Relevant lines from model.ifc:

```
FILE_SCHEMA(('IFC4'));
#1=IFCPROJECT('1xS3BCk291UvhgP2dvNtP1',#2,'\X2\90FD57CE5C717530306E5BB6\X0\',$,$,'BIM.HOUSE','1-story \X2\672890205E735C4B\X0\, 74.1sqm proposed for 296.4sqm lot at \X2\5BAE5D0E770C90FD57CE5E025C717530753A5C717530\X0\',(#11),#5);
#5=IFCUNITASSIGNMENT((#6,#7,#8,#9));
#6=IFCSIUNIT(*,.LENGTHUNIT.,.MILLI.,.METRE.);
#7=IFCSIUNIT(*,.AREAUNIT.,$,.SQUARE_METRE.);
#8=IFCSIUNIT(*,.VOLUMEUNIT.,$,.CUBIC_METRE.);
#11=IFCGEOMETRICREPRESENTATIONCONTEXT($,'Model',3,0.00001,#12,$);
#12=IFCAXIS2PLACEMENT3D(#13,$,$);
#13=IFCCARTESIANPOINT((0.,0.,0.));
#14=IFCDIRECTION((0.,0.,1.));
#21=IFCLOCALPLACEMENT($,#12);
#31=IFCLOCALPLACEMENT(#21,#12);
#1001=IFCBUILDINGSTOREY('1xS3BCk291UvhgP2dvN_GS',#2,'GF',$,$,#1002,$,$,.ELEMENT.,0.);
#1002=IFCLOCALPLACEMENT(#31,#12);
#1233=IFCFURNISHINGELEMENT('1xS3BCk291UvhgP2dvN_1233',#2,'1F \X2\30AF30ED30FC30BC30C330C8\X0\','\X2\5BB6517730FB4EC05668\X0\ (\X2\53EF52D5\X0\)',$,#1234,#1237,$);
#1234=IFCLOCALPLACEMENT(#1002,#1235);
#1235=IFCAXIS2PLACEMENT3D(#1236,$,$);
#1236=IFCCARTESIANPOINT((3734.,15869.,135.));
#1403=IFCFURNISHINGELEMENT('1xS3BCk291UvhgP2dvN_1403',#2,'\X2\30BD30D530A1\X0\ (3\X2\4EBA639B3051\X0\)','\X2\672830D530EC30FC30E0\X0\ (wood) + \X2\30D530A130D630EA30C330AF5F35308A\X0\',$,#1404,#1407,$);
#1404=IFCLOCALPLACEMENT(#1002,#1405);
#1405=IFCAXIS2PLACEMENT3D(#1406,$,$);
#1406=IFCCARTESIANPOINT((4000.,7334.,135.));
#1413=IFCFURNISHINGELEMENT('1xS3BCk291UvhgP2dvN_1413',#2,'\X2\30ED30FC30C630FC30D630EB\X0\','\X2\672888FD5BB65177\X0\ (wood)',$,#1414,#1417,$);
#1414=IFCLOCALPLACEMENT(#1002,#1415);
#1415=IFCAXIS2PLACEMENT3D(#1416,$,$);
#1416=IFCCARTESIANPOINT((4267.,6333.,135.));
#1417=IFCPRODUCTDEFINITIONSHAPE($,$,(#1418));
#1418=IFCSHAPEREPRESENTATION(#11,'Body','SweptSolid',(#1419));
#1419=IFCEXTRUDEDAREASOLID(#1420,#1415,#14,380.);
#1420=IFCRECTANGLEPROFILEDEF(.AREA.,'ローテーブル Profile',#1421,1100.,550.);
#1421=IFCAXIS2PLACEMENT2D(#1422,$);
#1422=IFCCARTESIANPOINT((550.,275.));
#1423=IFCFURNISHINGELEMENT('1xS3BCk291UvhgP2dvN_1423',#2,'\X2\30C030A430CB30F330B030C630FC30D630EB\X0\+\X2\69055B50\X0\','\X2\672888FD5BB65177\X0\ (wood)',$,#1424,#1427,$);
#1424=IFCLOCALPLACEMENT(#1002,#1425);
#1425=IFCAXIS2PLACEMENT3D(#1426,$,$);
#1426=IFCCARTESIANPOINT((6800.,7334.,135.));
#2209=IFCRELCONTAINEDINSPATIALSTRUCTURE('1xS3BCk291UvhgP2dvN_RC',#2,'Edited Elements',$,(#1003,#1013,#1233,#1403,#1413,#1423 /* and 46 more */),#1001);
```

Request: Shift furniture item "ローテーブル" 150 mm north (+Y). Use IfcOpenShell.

```python
import ifcopenshell
import ifcopenshell.api.geometry
import ifcopenshell.util.placement

model = ifcopenshell.open("model.ifc")

item = model.by_guid("1xS3BCk291UvhgP2dvN_1413")
matrix = ifcopenshell.util.placement.get_local_placement(item.ObjectPlacement)
matrix[1, 3] += 150.0
ifcopenshell.api.geometry.edit_object_placement(model, product=item, matrix=matrix, is_si=False)

print(ifcopenshell.util.placement.get_local_placement(item.ObjectPlacement).round(3) + 0.0)

model.write("model-out.ifc")
```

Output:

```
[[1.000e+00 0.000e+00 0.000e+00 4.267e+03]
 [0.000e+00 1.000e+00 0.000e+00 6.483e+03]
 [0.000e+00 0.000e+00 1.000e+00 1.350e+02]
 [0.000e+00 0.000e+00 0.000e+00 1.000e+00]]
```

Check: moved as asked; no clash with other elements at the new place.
